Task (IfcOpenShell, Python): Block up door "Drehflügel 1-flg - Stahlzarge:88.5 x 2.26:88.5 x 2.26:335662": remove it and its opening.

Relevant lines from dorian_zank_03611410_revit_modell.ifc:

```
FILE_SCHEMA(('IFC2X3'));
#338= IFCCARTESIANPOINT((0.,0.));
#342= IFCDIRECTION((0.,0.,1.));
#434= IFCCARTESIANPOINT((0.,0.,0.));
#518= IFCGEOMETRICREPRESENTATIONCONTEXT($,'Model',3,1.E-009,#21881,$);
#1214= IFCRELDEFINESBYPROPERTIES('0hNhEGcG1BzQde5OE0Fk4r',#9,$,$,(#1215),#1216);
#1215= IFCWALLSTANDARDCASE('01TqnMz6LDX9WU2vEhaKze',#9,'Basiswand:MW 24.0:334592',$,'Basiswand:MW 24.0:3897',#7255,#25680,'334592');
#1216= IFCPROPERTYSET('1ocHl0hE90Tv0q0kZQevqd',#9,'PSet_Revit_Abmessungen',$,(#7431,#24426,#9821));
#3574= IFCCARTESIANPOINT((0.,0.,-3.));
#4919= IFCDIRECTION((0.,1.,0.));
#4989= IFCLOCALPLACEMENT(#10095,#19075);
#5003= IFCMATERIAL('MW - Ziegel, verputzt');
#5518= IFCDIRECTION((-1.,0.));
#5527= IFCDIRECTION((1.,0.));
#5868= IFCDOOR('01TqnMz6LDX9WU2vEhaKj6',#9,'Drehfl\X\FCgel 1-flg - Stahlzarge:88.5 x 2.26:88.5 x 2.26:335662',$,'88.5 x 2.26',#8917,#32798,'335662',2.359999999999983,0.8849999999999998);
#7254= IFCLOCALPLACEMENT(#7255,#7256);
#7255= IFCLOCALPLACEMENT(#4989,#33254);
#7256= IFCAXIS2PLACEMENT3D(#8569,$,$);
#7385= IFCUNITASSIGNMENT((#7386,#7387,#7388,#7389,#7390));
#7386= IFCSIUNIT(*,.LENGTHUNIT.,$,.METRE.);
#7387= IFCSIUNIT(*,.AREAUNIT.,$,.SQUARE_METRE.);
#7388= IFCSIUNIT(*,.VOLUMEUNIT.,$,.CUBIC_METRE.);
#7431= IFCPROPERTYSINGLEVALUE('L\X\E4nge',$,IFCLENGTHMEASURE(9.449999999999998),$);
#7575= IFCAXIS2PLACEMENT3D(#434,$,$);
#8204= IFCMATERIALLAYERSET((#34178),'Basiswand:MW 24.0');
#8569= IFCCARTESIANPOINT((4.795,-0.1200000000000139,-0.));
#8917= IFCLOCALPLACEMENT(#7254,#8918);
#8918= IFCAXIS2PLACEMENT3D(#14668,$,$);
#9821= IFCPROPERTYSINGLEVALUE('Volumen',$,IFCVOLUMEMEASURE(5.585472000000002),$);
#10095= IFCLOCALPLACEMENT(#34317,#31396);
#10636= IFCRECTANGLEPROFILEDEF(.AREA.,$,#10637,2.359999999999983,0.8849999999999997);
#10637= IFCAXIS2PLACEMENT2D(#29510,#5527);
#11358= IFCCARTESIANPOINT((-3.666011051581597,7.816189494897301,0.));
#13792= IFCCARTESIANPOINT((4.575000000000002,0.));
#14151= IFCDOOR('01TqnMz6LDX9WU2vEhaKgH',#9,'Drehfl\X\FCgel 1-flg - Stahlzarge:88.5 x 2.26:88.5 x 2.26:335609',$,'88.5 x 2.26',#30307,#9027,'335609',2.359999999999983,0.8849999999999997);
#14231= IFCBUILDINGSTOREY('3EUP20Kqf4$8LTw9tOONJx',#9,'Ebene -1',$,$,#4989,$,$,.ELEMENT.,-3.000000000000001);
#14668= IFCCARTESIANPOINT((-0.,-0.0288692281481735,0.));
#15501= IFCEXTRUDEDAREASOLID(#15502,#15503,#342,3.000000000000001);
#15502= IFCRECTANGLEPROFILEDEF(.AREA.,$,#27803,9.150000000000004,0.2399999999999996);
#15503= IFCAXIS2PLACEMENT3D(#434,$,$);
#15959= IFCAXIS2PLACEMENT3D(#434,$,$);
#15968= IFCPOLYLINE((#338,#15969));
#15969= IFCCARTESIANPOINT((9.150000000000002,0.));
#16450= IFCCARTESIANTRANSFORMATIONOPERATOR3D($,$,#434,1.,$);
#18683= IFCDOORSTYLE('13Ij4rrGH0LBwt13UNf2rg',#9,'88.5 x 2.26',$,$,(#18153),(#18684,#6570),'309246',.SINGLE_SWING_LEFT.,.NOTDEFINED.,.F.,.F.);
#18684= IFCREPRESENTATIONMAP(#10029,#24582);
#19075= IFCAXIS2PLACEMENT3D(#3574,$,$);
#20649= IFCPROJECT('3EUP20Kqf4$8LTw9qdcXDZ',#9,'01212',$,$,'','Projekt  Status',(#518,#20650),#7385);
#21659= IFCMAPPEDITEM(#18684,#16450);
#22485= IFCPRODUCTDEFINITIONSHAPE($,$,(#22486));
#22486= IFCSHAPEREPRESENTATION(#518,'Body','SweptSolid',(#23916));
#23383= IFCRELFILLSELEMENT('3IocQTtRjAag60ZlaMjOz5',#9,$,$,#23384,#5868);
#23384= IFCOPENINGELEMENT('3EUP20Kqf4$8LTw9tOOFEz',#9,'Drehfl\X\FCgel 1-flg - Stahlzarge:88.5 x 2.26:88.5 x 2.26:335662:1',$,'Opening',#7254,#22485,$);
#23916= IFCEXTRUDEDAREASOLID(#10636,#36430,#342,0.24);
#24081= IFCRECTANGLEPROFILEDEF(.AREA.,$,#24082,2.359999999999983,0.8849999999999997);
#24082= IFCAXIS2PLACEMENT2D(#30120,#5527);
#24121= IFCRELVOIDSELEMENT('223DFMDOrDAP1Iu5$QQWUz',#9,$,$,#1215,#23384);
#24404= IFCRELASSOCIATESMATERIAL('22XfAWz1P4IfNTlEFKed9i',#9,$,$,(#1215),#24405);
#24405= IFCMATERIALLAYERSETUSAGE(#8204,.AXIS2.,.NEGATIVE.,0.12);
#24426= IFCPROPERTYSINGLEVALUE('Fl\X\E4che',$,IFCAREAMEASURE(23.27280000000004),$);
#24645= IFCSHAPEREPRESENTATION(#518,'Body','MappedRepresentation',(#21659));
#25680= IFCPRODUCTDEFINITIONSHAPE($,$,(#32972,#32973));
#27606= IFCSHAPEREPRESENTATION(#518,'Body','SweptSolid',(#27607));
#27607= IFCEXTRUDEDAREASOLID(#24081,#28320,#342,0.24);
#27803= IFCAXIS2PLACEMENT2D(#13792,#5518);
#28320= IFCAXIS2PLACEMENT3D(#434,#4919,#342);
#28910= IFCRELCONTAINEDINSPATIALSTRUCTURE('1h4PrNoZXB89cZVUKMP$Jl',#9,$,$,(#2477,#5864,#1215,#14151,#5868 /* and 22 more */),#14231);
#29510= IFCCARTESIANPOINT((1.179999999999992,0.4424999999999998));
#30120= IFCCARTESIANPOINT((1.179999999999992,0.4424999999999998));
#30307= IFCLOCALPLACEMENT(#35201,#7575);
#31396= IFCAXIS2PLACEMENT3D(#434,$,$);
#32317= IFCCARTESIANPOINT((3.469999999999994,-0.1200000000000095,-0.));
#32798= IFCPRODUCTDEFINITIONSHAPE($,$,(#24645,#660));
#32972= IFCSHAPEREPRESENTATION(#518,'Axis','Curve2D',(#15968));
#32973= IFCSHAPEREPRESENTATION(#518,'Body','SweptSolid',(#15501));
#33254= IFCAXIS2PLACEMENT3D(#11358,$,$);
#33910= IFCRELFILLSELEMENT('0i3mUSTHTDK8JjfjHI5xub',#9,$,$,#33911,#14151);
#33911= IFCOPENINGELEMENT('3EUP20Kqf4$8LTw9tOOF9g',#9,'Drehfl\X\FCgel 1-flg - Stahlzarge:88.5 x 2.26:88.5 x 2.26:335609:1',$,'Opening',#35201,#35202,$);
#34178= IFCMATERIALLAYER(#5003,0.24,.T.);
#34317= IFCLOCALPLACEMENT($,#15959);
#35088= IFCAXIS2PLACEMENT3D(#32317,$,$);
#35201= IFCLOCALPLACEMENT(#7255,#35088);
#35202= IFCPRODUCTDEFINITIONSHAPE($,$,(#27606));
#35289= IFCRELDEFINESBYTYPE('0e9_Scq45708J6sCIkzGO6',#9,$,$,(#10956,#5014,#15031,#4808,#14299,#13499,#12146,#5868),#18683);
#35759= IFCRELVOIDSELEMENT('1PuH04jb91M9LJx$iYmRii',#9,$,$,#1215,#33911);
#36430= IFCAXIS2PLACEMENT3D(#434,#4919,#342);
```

```python
import ifcopenshell
import ifcopenshell.api.feature
import ifcopenshell.api.pset
import ifcopenshell.api.root
import ifcopenshell.geom
import ifcopenshell.util.element
import ifcopenshell.util.shape
import ifcopenshell.util.unit

model = ifcopenshell.open("dorian_zank_03611410_revit_modell.ifc")
area_scale = ifcopenshell.util.unit.calculate_unit_scale(model, "AREAUNIT")
volume_scale = ifcopenshell.util.unit.calculate_unit_scale(model, "VOLUMEUNIT")
settings = ifcopenshell.geom.settings()


def volume(element):
    """Net volume in cubic metres, openings subtracted."""
    shape = ifcopenshell.geom.create_shape(settings, element)
    return ifcopenshell.util.shape.get_volume(shape.geometry)


door = model.by_guid("01TqnMz6LDX9WU2vEhaKj6")
opening = door.FillsVoids[0].RelatingOpeningElement
wall = opening.VoidsElements[0].RelatingBuildingElement
before = volume(wall)

ifcopenshell.api.root.remove_product(model, product=door)
ifcopenshell.api.feature.remove_feature(model, feature=opening)

after = volume(wall)
thickness = 0.24  # wall thickness in metres

# Update the wall's stored quantities.
pset = model.by_id(ifcopenshell.util.element.get_pset(wall, "PSet_Revit_Abmessungen", should_inherit=False)["id"])
ifcopenshell.api.pset.edit_pset(model, pset=pset, properties={
    "Fläche": model.create_entity("IfcAreaMeasure", after / thickness / area_scale),
    "Volumen": model.create_entity("IfcVolumeMeasure", after / volume_scale),
})

print(f"wall volume {before:.3f} -> {after:.3f} m3")

model.write("dorian_zank_03611410_revit_modell-out.ifc")
```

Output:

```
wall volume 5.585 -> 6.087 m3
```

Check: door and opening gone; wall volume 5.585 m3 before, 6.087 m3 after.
